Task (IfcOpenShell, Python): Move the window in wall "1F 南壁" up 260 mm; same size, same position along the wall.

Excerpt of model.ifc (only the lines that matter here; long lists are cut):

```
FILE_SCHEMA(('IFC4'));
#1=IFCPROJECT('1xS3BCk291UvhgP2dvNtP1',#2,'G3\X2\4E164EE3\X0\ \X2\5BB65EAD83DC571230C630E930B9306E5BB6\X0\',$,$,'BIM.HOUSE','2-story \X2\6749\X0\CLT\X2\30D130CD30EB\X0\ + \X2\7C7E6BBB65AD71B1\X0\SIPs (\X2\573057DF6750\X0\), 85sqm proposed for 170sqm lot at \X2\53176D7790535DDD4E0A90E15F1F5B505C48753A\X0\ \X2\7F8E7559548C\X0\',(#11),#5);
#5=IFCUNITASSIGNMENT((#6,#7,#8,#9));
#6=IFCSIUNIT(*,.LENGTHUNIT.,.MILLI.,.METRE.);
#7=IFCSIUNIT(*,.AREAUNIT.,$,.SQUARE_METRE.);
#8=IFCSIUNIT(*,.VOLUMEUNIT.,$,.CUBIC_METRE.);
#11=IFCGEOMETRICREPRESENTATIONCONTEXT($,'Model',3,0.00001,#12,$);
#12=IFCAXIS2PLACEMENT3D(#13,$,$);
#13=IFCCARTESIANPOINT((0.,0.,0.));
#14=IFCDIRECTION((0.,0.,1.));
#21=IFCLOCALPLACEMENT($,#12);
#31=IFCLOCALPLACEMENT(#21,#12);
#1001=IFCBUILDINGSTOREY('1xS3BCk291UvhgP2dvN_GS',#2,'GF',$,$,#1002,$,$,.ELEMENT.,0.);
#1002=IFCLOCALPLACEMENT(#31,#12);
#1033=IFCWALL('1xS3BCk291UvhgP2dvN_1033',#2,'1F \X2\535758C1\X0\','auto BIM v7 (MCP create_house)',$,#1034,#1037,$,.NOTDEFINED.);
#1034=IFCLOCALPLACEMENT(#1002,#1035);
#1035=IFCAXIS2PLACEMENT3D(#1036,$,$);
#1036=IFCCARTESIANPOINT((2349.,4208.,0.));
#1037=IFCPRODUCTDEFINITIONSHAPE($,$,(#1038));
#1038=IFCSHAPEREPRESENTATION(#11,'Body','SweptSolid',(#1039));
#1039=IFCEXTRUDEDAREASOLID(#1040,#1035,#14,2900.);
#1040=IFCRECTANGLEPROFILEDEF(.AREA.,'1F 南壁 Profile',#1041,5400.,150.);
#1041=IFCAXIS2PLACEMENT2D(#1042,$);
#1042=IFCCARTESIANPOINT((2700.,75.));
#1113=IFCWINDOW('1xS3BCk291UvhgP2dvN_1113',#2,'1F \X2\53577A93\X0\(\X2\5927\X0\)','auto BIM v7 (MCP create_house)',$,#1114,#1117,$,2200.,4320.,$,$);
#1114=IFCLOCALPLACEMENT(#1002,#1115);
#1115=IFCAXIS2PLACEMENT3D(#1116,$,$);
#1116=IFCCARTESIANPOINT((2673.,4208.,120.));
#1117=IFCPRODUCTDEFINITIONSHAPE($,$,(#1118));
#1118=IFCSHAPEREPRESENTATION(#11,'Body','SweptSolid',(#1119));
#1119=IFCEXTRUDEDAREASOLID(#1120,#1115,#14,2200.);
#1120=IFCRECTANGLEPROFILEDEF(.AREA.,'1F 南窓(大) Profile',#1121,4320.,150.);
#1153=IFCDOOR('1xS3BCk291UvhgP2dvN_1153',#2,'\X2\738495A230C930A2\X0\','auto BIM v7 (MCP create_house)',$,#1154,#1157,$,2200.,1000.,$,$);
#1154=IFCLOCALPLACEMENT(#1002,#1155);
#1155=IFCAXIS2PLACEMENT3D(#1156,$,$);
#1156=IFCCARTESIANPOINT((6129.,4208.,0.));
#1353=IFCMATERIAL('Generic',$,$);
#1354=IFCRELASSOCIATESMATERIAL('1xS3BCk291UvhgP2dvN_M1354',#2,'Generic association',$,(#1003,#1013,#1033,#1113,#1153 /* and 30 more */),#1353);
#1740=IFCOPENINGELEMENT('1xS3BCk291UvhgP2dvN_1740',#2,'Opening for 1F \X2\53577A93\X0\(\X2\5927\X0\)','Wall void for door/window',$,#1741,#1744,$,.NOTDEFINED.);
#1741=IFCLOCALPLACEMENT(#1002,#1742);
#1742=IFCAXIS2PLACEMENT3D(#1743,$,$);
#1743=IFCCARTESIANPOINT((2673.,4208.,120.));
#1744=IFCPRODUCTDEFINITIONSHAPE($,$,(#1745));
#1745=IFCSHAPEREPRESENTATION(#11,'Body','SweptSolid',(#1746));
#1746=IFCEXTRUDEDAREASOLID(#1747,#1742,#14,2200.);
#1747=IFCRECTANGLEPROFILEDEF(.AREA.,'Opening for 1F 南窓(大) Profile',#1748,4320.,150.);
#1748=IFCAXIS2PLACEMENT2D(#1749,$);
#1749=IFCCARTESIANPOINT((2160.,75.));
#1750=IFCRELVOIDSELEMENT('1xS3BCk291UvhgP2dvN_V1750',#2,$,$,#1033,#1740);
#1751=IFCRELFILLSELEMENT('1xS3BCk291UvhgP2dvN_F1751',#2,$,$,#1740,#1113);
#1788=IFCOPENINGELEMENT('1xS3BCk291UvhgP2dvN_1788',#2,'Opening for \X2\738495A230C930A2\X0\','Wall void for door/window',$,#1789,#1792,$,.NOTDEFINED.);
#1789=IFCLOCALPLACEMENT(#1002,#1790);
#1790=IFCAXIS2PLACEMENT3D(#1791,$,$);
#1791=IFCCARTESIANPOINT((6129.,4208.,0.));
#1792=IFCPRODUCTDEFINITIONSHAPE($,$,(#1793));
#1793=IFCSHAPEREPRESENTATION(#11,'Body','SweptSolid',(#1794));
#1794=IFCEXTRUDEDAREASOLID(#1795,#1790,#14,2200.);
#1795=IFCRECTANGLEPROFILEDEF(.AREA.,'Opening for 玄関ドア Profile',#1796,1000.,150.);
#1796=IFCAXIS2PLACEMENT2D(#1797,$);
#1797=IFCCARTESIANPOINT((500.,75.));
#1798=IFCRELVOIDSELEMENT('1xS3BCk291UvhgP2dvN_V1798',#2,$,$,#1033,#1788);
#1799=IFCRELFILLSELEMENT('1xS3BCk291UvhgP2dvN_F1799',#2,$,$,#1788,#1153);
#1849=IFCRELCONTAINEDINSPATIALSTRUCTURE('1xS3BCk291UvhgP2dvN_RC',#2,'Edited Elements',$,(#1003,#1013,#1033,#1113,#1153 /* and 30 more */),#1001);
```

```python
import numpy as np
import ifcopenshell
import ifcopenshell.api.geometry
import ifcopenshell.util.placement
import ifcopenshell.util.unit

model = ifcopenshell.open("model.ifc")
unit_scale = ifcopenshell.util.unit.calculate_unit_scale(model)

window = model.by_guid("1xS3BCk291UvhgP2dvN_1113")
opening = window.FillsVoids[0].RelatingOpeningElement
dz = 260.0

shift = np.array([0.0, 0.0, dz])
# The window is not placed relative to its opening, so move both.
for product in (opening, window):
    matrix = ifcopenshell.util.placement.get_local_placement(product.ObjectPlacement)
    matrix[:3, 3] += shift
    ifcopenshell.api.geometry.edit_object_placement(model, product=product, matrix=matrix, is_si=False)

print(f"moved by {dz * unit_scale:+.3f} m")

model.write("model_edited.ifc")
```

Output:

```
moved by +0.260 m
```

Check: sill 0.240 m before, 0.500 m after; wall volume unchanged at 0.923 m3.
